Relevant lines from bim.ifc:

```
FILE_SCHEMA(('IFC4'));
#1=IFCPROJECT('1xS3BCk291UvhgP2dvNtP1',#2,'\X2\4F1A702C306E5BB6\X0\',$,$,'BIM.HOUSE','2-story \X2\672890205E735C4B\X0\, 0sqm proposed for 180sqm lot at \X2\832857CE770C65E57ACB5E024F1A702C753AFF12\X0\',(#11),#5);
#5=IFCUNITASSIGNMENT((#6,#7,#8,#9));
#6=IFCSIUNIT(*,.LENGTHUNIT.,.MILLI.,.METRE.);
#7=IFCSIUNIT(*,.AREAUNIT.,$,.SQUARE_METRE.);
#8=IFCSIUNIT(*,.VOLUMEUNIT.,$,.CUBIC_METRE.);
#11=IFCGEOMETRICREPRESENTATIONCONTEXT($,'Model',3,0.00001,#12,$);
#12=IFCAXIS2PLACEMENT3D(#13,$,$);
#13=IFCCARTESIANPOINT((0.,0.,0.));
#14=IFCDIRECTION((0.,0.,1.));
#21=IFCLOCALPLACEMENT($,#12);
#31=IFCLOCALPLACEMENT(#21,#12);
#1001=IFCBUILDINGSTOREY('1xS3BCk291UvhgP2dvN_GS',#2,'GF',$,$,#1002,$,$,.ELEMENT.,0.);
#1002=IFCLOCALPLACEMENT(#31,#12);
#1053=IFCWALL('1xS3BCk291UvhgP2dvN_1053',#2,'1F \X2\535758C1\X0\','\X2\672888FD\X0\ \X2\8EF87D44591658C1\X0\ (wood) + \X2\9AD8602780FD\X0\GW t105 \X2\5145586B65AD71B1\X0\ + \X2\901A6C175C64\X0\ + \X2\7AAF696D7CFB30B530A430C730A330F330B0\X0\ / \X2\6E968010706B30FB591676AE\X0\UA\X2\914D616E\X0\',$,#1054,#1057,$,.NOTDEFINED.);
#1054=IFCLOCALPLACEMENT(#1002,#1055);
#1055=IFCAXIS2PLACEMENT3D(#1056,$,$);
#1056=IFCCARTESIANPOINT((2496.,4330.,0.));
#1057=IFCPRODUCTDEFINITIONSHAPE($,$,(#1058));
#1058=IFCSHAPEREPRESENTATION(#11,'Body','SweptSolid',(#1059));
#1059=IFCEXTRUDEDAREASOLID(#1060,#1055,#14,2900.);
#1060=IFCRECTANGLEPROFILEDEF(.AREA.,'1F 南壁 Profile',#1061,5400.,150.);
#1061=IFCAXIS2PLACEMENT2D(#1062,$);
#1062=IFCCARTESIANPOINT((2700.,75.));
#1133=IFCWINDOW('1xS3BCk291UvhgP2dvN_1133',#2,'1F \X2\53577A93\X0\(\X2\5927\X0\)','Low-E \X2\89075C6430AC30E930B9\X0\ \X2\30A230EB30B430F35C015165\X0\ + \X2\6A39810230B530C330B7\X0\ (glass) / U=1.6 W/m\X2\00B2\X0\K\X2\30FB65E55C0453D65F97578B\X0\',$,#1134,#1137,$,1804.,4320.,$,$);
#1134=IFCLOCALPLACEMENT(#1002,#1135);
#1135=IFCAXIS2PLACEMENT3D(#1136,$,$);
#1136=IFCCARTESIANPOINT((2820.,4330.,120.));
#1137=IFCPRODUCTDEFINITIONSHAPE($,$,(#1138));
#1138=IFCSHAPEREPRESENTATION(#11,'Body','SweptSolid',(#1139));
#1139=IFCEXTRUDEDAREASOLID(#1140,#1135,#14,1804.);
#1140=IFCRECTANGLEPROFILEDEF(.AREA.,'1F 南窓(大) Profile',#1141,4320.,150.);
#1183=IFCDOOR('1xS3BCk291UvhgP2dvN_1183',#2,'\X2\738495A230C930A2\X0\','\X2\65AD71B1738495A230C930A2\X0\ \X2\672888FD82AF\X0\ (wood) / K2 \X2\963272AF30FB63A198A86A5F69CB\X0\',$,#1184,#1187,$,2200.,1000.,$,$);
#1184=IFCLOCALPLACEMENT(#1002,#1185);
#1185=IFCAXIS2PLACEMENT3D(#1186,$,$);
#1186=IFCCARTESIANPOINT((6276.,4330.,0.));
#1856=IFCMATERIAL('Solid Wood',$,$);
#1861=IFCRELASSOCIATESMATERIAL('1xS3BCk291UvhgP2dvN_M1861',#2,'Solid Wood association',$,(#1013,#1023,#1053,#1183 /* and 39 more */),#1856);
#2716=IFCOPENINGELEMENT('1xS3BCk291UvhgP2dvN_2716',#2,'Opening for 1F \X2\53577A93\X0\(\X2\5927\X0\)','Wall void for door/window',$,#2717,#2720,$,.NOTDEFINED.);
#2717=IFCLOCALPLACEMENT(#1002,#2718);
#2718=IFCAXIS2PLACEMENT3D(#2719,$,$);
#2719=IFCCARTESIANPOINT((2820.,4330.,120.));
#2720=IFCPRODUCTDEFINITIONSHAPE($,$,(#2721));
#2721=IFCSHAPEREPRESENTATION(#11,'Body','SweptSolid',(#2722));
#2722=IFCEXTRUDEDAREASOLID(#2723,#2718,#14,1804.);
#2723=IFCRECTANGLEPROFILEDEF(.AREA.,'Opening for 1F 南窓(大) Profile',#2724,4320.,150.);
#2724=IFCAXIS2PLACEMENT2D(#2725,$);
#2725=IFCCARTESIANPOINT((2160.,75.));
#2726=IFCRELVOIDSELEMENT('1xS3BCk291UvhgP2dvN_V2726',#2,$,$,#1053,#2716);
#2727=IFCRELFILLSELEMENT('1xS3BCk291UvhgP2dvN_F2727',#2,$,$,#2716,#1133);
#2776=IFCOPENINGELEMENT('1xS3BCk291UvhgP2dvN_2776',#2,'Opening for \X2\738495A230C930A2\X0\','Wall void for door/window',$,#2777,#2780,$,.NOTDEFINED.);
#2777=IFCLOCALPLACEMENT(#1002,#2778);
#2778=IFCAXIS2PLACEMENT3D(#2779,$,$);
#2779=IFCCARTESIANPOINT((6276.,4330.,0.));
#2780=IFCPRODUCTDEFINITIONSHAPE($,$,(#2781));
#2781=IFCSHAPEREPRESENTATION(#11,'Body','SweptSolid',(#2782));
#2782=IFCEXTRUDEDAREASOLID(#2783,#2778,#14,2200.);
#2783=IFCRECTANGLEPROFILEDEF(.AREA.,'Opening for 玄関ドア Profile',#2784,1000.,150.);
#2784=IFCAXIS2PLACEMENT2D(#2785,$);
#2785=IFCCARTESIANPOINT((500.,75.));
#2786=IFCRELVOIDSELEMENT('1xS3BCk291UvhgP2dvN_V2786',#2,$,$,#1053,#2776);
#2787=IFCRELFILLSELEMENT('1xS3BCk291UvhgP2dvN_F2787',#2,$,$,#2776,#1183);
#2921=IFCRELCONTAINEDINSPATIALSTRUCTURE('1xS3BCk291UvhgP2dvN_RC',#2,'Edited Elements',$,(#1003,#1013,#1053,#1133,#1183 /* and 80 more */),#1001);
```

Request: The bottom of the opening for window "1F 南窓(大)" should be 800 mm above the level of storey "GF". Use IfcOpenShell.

```python
import numpy as np
import ifcopenshell
import ifcopenshell.api.geometry
import ifcopenshell.geom
import ifcopenshell.util.element
import ifcopenshell.util.placement
import ifcopenshell.util.shape
import ifcopenshell.util.unit

model = ifcopenshell.open("bim.ifc")
unit_scale = ifcopenshell.util.unit.calculate_unit_scale(model)

window = model.by_id(1133)
opening = window.FillsVoids[0].RelatingOpeningElement
storey = ifcopenshell.util.element.get_container(window, ifc_class="IfcBuildingStorey")
level = ifcopenshell.util.placement.get_local_placement(storey.ObjectPlacement)[2, 3]

# The opening's origin need not be at the sill, so measure its lowest point.
shape = ifcopenshell.geom.create_shape(ifcopenshell.geom.settings(), opening)
bottom = ifcopenshell.util.shape.get_shape_bottom_elevation(shape, shape.geometry) / unit_scale
dz = level + 0.8 / unit_scale - bottom

shift = np.array([0.0, 0.0, dz])
# The window is not placed relative to its opening, so move both.
for product in (opening, window):
    matrix = ifcopenshell.util.placement.get_local_placement(product.ObjectPlacement)
    matrix[:3, 3] += shift
    ifcopenshell.api.geometry.edit_object_placement(model, product=product, matrix=matrix, is_si=False)

print(f"moved by {dz * unit_scale:+.3f} m")

model.write("bim-out.ifc")
```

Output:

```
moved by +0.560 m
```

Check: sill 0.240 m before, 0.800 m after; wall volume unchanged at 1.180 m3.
